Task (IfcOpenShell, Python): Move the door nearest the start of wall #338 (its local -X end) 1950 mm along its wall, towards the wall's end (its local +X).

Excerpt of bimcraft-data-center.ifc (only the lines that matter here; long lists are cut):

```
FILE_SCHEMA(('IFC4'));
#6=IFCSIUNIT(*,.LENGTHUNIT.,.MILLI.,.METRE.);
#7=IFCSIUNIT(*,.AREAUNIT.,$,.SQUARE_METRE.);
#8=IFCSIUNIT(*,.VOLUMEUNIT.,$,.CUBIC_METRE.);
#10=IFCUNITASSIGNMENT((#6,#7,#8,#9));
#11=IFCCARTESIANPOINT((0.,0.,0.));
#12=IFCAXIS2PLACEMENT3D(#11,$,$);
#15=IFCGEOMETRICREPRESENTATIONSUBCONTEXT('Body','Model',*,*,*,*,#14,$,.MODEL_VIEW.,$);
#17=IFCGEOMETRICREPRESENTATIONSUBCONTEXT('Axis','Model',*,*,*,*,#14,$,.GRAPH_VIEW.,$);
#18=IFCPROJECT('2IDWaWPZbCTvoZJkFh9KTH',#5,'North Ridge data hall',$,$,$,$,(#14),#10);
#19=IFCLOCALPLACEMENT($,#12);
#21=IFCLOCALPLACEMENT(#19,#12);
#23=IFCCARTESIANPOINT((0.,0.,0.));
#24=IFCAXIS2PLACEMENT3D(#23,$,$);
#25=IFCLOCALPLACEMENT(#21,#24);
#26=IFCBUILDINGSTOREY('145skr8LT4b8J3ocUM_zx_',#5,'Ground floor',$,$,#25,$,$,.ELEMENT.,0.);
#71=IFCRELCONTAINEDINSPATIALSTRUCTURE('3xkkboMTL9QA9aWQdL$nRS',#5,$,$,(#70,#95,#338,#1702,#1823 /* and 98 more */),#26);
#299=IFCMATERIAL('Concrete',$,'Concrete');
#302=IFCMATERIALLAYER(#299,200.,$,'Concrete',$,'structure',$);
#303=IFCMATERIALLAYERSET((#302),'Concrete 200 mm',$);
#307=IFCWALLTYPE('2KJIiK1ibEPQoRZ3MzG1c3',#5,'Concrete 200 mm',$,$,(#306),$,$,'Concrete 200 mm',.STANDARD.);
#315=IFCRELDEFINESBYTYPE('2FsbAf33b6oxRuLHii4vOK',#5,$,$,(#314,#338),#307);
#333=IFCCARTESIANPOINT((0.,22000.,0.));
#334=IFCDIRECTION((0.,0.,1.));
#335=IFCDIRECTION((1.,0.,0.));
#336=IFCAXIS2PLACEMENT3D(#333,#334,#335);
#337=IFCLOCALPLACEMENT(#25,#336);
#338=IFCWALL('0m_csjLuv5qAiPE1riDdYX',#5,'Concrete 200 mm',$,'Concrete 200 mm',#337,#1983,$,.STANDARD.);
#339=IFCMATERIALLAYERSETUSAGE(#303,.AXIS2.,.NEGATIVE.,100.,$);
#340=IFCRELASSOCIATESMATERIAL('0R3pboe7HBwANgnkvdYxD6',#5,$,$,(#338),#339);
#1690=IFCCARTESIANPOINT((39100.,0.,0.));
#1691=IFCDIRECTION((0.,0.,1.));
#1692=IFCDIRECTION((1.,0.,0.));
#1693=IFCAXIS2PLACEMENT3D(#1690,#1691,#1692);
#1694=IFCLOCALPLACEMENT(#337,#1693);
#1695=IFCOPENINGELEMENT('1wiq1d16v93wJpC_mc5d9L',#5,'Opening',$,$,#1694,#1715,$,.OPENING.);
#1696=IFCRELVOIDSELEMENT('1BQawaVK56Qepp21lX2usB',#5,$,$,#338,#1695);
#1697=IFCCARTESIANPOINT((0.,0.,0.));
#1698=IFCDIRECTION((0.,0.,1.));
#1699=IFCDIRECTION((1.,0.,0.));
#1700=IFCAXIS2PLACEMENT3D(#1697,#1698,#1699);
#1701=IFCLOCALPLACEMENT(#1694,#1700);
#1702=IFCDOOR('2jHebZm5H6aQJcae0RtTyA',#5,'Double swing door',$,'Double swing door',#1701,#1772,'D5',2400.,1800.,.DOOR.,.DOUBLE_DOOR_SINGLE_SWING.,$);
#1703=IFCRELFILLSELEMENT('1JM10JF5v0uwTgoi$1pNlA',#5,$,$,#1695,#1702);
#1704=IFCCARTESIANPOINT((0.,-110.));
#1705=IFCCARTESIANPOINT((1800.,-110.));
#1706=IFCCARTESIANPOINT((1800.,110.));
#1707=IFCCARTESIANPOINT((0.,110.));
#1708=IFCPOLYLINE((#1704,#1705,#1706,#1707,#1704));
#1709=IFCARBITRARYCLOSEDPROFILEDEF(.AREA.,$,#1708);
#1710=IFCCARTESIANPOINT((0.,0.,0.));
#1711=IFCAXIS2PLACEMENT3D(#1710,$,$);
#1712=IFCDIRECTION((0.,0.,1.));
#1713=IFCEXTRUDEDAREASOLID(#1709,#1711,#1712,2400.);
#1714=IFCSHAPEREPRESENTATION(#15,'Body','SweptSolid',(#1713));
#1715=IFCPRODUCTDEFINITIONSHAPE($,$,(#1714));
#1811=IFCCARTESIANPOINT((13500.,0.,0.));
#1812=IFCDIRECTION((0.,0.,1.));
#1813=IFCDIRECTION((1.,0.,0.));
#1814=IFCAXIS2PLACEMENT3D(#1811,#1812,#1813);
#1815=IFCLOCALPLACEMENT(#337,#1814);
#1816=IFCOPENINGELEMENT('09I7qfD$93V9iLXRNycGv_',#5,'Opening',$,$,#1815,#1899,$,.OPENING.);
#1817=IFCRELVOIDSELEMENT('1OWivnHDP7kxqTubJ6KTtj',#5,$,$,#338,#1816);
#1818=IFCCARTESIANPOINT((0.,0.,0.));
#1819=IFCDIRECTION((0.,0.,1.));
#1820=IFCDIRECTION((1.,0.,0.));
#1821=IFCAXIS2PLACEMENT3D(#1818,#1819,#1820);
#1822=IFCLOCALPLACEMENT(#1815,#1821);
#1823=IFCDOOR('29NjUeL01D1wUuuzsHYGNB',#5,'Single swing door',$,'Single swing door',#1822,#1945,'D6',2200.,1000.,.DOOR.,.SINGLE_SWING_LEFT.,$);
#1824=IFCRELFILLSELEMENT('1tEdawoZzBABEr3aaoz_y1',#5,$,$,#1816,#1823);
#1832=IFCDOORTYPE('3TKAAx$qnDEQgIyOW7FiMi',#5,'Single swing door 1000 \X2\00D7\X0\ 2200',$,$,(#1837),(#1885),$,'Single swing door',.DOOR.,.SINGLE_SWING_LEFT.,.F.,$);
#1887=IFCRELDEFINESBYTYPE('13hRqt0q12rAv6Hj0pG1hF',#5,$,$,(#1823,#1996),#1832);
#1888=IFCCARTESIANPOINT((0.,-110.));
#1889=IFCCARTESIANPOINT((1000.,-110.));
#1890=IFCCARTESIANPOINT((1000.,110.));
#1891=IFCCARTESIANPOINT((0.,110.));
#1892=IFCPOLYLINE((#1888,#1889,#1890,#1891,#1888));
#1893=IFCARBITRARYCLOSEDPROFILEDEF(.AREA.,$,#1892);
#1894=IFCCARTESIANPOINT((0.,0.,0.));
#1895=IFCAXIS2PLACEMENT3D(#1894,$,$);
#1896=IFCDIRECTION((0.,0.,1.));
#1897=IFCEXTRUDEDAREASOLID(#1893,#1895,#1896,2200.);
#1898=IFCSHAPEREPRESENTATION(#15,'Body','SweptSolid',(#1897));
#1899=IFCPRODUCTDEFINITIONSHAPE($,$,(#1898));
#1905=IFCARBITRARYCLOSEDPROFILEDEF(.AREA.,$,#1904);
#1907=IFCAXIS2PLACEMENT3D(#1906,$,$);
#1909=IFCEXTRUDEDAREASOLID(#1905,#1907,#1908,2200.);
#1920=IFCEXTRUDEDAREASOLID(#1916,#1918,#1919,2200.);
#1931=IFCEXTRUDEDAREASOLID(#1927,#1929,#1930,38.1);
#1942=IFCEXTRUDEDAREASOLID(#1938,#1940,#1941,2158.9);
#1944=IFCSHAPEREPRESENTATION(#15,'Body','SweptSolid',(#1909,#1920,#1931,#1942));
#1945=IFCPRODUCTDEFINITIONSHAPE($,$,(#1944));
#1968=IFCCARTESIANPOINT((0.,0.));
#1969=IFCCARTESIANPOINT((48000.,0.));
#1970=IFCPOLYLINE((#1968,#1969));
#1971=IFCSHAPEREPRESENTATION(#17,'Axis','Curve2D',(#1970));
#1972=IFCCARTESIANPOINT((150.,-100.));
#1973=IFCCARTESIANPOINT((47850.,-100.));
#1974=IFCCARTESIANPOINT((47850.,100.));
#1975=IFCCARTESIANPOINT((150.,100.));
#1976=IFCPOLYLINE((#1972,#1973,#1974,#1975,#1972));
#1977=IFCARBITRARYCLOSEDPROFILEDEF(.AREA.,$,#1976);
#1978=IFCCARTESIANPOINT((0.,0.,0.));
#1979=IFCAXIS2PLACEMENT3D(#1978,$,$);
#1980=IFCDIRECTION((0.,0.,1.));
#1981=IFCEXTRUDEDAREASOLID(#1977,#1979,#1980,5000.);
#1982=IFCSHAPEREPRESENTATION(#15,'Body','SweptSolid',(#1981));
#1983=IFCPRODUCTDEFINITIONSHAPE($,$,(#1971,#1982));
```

```python
import ifcopenshell
import ifcopenshell.api.geometry
import ifcopenshell.util.placement

model = ifcopenshell.open("bimcraft-data-center.ifc")

door = model.by_guid("29NjUeL01D1wUuuzsHYGNB")
opening = door.FillsVoids[0].RelatingOpeningElement
wall = opening.VoidsElements[0].RelatingBuildingElement

wall_matrix = ifcopenshell.util.placement.get_local_placement(wall.ObjectPlacement)
shift = wall_matrix[:3, 0] * 1950.0
before = ifcopenshell.util.placement.get_local_placement(door.ObjectPlacement)[:3, 3].copy()

# The door is placed relative to its opening, so it follows when the opening moves.
matrix = ifcopenshell.util.placement.get_local_placement(opening.ObjectPlacement)
matrix[:3, 3] += shift
ifcopenshell.api.geometry.edit_object_placement(
    model, product=opening, matrix=matrix, is_si=False, should_transform_children=True
)

after = ifcopenshell.util.placement.get_local_placement(door.ObjectPlacement)[:3, 3]
print("door moved by", (after - before).round(3) + 0.0)

model.write("bimcraft-data-center_edited.ifc")
```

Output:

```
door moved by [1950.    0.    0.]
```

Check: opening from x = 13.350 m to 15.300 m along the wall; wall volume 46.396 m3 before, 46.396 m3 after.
